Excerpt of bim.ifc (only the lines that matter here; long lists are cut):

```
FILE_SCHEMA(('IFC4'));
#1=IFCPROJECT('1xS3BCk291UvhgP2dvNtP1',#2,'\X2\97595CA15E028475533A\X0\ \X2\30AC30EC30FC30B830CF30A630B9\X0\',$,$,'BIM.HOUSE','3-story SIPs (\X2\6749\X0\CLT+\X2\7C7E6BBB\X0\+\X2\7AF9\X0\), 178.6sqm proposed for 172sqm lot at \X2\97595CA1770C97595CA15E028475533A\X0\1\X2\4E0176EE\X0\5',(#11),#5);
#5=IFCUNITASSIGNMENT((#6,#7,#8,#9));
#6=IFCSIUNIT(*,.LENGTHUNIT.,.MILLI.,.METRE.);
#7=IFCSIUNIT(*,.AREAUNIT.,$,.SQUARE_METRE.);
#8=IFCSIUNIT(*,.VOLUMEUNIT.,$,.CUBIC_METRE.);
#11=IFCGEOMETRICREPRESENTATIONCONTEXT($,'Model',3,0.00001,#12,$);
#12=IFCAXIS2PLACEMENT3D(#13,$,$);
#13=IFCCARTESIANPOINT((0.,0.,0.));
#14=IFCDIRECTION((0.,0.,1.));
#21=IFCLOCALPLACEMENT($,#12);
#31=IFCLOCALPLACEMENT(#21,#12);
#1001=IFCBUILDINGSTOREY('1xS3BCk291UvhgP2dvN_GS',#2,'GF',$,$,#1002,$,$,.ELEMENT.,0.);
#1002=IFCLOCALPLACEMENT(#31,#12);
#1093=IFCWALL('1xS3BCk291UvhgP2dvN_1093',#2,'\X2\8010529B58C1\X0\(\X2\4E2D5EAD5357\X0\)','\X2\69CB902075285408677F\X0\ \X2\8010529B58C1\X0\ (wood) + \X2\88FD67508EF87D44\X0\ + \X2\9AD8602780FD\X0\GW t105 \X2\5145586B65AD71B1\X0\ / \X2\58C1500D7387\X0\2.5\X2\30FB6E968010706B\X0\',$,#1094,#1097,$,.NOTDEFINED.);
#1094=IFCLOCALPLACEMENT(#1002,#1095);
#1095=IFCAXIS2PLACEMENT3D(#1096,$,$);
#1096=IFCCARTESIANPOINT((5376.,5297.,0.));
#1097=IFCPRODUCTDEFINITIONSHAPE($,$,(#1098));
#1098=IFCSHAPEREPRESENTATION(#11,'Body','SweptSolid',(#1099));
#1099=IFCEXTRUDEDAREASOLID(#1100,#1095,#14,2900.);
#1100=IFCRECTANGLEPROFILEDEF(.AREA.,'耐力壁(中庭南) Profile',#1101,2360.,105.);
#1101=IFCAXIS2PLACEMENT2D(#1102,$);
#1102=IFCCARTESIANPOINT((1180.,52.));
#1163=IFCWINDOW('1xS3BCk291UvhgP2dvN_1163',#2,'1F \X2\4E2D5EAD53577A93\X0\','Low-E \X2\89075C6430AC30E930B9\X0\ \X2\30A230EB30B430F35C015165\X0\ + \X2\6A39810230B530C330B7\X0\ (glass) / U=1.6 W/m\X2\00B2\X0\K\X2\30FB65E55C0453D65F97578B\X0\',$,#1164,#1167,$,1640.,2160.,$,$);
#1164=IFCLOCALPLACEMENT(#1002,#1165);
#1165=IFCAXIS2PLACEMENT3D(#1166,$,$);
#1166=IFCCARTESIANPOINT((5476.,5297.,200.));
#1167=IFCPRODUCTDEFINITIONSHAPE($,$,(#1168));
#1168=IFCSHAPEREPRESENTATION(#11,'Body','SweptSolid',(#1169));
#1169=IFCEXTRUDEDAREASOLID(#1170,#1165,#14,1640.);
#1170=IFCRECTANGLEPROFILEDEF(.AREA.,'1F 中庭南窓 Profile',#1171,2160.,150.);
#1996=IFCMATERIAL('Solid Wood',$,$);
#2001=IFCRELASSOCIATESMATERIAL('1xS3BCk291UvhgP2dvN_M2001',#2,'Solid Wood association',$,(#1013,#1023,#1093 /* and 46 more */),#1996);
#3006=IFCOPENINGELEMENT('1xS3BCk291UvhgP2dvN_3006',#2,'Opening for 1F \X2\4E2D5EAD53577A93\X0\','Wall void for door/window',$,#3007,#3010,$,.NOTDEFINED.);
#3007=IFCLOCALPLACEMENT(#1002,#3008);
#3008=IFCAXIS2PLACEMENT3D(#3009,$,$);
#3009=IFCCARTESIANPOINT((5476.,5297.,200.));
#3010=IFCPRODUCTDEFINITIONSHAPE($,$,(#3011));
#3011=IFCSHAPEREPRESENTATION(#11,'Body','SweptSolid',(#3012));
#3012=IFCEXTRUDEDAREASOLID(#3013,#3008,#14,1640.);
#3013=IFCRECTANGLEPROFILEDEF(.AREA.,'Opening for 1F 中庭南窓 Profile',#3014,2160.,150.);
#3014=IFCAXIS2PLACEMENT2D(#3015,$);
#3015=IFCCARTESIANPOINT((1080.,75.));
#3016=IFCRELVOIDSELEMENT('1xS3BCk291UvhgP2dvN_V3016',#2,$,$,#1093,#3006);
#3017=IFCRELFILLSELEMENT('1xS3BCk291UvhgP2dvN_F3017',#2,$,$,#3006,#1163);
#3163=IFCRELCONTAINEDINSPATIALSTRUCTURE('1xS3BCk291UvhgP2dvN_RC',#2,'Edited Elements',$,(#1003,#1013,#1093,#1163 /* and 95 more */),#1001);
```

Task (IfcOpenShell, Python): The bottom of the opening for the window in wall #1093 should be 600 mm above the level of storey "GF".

```python
import numpy as np
import ifcopenshell
import ifcopenshell.api.geometry
import ifcopenshell.geom
import ifcopenshell.util.element
import ifcopenshell.util.placement
import ifcopenshell.util.shape
import ifcopenshell.util.unit

model = ifcopenshell.open("bim.ifc")
unit_scale = ifcopenshell.util.unit.calculate_unit_scale(model)

window = model.by_guid("1xS3BCk291UvhgP2dvN_1163")
opening = window.FillsVoids[0].RelatingOpeningElement
storey = ifcopenshell.util.element.get_container(window, ifc_class="IfcBuildingStorey")
level = ifcopenshell.util.placement.get_local_placement(storey.ObjectPlacement)[2, 3]

# The opening's origin need not be at the sill, so measure its lowest point.
shape = ifcopenshell.geom.create_shape(ifcopenshell.geom.settings(), opening)
bottom = ifcopenshell.util.shape.get_shape_bottom_elevation(shape, shape.geometry) / unit_scale
dz = level + 0.6 / unit_scale - bottom

shift = np.array([0.0, 0.0, dz])
# The window is not placed relative to its opening, so move both.
for product in (opening, window):
    matrix = ifcopenshell.util.placement.get_local_placement(product.ObjectPlacement)
    matrix[:3, 3] += shift
    ifcopenshell.api.geometry.edit_object_placement(model, product=product, matrix=matrix, is_si=False)

print(f"moved by {dz * unit_scale:+.3f} m")

model.write("bim_rev.ifc")
```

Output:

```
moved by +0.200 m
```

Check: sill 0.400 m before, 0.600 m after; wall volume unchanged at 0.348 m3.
